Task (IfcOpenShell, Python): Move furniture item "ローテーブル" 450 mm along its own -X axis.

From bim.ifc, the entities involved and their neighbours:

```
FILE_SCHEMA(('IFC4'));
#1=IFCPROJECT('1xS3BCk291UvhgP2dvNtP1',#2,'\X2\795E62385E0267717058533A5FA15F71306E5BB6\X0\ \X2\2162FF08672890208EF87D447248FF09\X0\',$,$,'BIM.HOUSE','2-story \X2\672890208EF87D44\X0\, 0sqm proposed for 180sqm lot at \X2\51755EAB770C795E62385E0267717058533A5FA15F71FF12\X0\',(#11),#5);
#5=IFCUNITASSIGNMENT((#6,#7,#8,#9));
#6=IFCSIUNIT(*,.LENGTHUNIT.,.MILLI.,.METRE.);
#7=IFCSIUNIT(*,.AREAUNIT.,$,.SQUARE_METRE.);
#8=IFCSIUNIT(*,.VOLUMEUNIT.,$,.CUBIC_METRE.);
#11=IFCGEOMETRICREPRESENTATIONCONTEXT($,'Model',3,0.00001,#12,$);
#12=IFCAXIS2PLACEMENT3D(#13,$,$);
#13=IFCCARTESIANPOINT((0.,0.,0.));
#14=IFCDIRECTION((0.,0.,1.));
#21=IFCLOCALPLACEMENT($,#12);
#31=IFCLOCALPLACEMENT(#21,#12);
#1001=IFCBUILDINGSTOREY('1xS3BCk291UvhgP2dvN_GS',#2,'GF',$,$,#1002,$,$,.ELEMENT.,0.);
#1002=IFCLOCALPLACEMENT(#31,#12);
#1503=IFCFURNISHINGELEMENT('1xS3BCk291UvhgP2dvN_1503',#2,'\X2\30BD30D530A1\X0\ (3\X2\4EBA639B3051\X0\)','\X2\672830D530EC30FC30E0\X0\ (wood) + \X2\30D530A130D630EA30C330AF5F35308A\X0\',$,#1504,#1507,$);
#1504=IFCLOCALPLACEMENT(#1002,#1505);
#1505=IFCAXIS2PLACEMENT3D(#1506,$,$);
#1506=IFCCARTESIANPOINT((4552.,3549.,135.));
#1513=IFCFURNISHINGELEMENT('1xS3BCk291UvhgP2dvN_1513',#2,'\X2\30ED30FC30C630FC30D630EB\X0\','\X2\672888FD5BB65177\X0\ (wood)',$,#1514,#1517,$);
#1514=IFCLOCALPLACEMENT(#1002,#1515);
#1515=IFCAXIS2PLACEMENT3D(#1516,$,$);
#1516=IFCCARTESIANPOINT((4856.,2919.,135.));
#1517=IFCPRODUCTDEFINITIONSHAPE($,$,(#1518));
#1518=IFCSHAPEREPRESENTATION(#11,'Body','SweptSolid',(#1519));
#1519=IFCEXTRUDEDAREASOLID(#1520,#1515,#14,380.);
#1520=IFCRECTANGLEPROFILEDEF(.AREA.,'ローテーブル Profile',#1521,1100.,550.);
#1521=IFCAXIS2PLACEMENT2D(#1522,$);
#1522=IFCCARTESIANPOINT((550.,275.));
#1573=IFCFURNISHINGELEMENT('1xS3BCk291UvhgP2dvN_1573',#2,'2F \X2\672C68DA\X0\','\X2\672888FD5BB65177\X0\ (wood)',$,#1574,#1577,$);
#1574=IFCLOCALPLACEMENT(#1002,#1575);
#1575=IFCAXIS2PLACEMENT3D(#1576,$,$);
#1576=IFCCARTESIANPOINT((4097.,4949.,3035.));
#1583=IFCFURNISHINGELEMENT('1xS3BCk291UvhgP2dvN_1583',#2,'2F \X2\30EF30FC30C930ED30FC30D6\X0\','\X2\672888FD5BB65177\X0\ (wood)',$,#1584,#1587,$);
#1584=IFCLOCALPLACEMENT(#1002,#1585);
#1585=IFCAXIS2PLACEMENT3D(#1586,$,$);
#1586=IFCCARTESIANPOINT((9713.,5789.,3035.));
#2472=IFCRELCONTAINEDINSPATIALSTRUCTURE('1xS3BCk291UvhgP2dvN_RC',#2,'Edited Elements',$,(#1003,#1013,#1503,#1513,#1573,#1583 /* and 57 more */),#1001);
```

```python
import ifcopenshell
import ifcopenshell.api.geometry
import ifcopenshell.util.placement

model = ifcopenshell.open("bim.ifc")

item = model.by_guid("1xS3BCk291UvhgP2dvN_1513")
matrix = ifcopenshell.util.placement.get_local_placement(item.ObjectPlacement)
matrix[:3, 3] -= matrix[:3, 0] * 450.0
ifcopenshell.api.geometry.edit_object_placement(model, product=item, matrix=matrix, is_si=False)

print(ifcopenshell.util.placement.get_local_placement(item.ObjectPlacement).round(3) + 0.0)

model.write("bim_v2.ifc")
```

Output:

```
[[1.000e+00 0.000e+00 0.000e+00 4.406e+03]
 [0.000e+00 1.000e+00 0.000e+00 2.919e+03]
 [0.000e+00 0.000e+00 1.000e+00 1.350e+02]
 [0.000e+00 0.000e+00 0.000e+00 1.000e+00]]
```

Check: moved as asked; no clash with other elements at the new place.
